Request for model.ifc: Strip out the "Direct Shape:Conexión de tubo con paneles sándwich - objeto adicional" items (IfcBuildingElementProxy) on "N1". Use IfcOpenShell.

First a look at what the model holds.

```python
import ifcopenshell
import ifcopenshell.util.element

model = ifcopenshell.open("model.ifc")
print(model.schema)
storey = next(s for s in model.by_type("IfcBuildingStorey") if s.Name == "N1")
proxies = [e for e in ifcopenshell.util.element.get_decomposition(storey) if e.is_a("IfcBuildingElementProxy")]
seen = {}
for e in proxies:
    element_type = ifcopenshell.util.element.get_type(e)
    name = element_type.Name if element_type not in (None, e) else None
    seen[name] = seen.get(name, 0) + 1
for name, count in sorted(seen.items(), key=str):
    print(count, "x", name)
```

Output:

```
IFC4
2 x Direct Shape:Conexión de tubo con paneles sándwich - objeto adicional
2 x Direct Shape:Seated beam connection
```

```python
import ifcopenshell
import ifcopenshell.api.root
import ifcopenshell.util.element

model = ifcopenshell.open("model.ifc")

storey = next(s for s in model.by_type("IfcBuildingStorey") if s.Name == "N1")
proxies = [e for e in ifcopenshell.util.element.get_decomposition(storey) if e.is_a("IfcBuildingElementProxy")]
targets = [e for e in proxies if (t := ifcopenshell.util.element.get_type(e)) not in (None, e) and t.Name == "Direct Shape:Conexión de tubo con paneles sándwich - objeto adicional"]

for e in targets:
    ifcopenshell.api.root.remove_product(model, product=e)
print(len(targets), "removed")

model.write("model_v2.ifc")
```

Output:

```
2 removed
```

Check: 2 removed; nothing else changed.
